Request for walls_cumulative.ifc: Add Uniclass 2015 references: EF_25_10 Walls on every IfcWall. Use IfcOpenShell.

First a look at what the model holds.

```python
import ifcopenshell

model = ifcopenshell.open("walls_cumulative.ifc")
print(model.schema)
print("classifications:", [c.Name for c in model.by_type("IfcClassification")])
for ifc_class in ("IfcDoor", "IfcRoof", "IfcStair", "IfcWall", "IfcWindow"):
    print(ifc_class, len(model.by_type(ifc_class)))
```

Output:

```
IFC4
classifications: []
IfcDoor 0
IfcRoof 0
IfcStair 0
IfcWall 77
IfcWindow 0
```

```python
import ifcopenshell
import ifcopenshell.api.classification

model = ifcopenshell.open("walls_cumulative.ifc")

system = ifcopenshell.api.classification.add_classification(model, classification="Uniclass 2015")

codes = {
    "IfcWall": ("EF_25_10", "Walls"),
}
for ifc_class, (code, name) in codes.items():
    products = model.by_type(ifc_class)
    ifcopenshell.api.classification.add_reference(
        model, products=products, classification=system, identification=code, name=name
    )
    print(code, len(products))

model.write("walls_cumulative_updated.ifc")
```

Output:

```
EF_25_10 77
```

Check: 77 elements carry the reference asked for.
